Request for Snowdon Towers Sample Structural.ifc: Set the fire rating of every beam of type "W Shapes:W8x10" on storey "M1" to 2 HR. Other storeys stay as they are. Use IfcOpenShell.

First a look at what the model holds.

```python
import ifcopenshell
import ifcopenshell.util.element

model = ifcopenshell.open("Snowdon Towers Sample Structural.ifc")
print(model.schema)
storey = next(s for s in model.by_type("IfcBuildingStorey") if s.Name == "M1")
beams = [e for e in ifcopenshell.util.element.get_decomposition(storey) if e.is_a("IfcBeam")]
seen = {}
for e in beams:
    element_type = ifcopenshell.util.element.get_type(e)
    key = (element_type.Name if element_type != e and element_type else None, ifcopenshell.util.element.get_pset(e, "Pset_BeamCommon", "FireRating"))
    seen[key] = seen.get(key, 0) + 1
for (name, value), count in sorted(seen.items(), key=str):
    print(count, "x", name, "|", value)
```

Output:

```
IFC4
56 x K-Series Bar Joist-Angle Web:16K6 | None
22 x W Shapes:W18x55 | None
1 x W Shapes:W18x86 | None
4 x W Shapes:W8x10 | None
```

```python
import ifcopenshell
import ifcopenshell.api.pset
import ifcopenshell.util.element

model = ifcopenshell.open("Snowdon Towers Sample Structural.ifc")

storey = next(s for s in model.by_type("IfcBuildingStorey") if s.Name == "M1")
beams = [e for e in ifcopenshell.util.element.get_decomposition(storey) if e.is_a("IfcBeam")]

count = 0
for e in beams:
    element_type = ifcopenshell.util.element.get_type(e)
    if element_type in (None, e) or element_type.Name != "W Shapes:W8x10":
        continue
    # add_pset returns the element's existing set when there is one.
    pset = ifcopenshell.api.pset.add_pset(model, product=e, name="Pset_BeamCommon")
    ifcopenshell.api.pset.edit_pset(model, pset=pset, properties={"FireRating": "2 HR"})
    count += 1

print(count, "beams updated")

model.write("Snowdon Towers Sample Structural_updated.ifc")
```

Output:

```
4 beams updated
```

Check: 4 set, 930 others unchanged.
